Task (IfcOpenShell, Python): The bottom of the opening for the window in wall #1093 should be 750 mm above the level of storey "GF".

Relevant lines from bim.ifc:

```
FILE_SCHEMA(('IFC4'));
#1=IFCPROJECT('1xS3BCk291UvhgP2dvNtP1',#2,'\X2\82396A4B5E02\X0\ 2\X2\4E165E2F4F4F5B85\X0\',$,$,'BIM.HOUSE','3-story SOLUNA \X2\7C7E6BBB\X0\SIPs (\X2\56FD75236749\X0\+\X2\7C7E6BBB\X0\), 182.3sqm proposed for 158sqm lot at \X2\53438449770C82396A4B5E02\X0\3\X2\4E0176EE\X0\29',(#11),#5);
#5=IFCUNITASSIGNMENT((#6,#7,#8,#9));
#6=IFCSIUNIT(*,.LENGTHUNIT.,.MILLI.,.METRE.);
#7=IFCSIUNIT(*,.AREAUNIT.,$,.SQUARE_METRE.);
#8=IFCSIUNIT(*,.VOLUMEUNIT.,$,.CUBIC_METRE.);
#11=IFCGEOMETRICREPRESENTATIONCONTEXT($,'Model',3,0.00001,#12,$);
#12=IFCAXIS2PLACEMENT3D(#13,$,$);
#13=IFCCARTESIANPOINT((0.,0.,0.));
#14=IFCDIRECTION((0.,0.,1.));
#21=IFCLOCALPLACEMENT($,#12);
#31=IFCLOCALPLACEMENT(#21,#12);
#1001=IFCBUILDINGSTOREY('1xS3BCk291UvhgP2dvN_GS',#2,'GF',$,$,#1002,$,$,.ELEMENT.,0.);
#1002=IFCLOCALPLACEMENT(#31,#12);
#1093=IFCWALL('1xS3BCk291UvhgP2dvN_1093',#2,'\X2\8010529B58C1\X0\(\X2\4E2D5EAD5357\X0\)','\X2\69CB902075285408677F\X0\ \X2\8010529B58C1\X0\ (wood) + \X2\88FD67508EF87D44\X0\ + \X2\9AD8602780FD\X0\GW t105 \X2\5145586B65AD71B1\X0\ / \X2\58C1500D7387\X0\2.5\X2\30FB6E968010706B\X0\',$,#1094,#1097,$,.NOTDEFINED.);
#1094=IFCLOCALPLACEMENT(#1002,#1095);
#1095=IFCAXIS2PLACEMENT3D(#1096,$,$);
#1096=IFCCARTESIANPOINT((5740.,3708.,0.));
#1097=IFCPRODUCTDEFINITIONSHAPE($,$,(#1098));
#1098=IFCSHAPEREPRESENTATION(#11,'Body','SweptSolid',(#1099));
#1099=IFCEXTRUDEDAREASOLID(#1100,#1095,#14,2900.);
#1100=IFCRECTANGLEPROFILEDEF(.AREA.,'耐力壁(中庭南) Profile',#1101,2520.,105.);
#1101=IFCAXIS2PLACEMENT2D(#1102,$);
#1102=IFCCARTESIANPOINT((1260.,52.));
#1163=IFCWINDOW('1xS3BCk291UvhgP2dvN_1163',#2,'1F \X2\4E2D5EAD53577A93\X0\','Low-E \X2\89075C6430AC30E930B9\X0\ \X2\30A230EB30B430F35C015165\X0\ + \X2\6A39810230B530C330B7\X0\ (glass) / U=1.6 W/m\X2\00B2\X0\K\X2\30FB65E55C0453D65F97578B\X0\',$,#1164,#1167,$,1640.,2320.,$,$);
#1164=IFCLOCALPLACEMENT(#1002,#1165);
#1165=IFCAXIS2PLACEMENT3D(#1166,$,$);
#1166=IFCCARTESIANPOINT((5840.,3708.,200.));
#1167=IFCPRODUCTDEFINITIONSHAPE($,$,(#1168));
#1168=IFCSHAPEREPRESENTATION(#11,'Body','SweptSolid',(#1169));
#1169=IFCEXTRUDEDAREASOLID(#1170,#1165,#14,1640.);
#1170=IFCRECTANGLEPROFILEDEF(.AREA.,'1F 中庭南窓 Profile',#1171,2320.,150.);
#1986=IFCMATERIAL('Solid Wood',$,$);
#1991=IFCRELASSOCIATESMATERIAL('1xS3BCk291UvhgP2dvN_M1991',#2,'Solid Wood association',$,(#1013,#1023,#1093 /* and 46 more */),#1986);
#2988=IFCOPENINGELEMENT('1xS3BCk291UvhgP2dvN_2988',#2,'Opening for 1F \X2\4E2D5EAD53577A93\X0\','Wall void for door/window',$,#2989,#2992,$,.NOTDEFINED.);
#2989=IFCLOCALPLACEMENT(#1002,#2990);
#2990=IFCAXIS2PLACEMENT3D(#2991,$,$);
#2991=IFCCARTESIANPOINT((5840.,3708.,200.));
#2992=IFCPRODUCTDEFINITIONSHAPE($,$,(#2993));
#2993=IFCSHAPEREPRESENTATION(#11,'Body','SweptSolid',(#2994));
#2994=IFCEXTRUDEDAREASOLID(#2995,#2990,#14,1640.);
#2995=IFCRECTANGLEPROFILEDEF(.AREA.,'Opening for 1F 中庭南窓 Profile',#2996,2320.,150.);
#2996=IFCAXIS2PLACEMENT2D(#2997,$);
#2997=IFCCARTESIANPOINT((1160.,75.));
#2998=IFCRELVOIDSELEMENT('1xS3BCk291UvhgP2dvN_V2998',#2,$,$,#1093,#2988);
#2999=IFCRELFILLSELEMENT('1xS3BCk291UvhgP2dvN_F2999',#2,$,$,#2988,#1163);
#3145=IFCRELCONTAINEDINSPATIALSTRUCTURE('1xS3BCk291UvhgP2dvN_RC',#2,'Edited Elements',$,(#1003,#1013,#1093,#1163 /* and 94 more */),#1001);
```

```python
import numpy as np
import ifcopenshell
import ifcopenshell.api.geometry
import ifcopenshell.geom
import ifcopenshell.util.element
import ifcopenshell.util.placement
import ifcopenshell.util.shape
import ifcopenshell.util.unit

model = ifcopenshell.open("bim.ifc")
unit_scale = ifcopenshell.util.unit.calculate_unit_scale(model)

window = model.by_guid("1xS3BCk291UvhgP2dvN_1163")
opening = window.FillsVoids[0].RelatingOpeningElement
storey = ifcopenshell.util.element.get_container(window, ifc_class="IfcBuildingStorey")
level = ifcopenshell.util.placement.get_local_placement(storey.ObjectPlacement)[2, 3]

# The opening's origin need not be at the sill, so measure its lowest point.
shape = ifcopenshell.geom.create_shape(ifcopenshell.geom.settings(), opening)
bottom = ifcopenshell.util.shape.get_shape_bottom_elevation(shape, shape.geometry) / unit_scale
dz = level + 0.75 / unit_scale - bottom

shift = np.array([0.0, 0.0, dz])
# The window is not placed relative to its opening, so move both.
for product in (opening, window):
    matrix = ifcopenshell.util.placement.get_local_placement(product.ObjectPlacement)
    matrix[:3, 3] += shift
    ifcopenshell.api.geometry.edit_object_placement(model, product=product, matrix=matrix, is_si=False)

print(f"moved by {dz * unit_scale:+.3f} m")

model.write("bim_updated.ifc")
```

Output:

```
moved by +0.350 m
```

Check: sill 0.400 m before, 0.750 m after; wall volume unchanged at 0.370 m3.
